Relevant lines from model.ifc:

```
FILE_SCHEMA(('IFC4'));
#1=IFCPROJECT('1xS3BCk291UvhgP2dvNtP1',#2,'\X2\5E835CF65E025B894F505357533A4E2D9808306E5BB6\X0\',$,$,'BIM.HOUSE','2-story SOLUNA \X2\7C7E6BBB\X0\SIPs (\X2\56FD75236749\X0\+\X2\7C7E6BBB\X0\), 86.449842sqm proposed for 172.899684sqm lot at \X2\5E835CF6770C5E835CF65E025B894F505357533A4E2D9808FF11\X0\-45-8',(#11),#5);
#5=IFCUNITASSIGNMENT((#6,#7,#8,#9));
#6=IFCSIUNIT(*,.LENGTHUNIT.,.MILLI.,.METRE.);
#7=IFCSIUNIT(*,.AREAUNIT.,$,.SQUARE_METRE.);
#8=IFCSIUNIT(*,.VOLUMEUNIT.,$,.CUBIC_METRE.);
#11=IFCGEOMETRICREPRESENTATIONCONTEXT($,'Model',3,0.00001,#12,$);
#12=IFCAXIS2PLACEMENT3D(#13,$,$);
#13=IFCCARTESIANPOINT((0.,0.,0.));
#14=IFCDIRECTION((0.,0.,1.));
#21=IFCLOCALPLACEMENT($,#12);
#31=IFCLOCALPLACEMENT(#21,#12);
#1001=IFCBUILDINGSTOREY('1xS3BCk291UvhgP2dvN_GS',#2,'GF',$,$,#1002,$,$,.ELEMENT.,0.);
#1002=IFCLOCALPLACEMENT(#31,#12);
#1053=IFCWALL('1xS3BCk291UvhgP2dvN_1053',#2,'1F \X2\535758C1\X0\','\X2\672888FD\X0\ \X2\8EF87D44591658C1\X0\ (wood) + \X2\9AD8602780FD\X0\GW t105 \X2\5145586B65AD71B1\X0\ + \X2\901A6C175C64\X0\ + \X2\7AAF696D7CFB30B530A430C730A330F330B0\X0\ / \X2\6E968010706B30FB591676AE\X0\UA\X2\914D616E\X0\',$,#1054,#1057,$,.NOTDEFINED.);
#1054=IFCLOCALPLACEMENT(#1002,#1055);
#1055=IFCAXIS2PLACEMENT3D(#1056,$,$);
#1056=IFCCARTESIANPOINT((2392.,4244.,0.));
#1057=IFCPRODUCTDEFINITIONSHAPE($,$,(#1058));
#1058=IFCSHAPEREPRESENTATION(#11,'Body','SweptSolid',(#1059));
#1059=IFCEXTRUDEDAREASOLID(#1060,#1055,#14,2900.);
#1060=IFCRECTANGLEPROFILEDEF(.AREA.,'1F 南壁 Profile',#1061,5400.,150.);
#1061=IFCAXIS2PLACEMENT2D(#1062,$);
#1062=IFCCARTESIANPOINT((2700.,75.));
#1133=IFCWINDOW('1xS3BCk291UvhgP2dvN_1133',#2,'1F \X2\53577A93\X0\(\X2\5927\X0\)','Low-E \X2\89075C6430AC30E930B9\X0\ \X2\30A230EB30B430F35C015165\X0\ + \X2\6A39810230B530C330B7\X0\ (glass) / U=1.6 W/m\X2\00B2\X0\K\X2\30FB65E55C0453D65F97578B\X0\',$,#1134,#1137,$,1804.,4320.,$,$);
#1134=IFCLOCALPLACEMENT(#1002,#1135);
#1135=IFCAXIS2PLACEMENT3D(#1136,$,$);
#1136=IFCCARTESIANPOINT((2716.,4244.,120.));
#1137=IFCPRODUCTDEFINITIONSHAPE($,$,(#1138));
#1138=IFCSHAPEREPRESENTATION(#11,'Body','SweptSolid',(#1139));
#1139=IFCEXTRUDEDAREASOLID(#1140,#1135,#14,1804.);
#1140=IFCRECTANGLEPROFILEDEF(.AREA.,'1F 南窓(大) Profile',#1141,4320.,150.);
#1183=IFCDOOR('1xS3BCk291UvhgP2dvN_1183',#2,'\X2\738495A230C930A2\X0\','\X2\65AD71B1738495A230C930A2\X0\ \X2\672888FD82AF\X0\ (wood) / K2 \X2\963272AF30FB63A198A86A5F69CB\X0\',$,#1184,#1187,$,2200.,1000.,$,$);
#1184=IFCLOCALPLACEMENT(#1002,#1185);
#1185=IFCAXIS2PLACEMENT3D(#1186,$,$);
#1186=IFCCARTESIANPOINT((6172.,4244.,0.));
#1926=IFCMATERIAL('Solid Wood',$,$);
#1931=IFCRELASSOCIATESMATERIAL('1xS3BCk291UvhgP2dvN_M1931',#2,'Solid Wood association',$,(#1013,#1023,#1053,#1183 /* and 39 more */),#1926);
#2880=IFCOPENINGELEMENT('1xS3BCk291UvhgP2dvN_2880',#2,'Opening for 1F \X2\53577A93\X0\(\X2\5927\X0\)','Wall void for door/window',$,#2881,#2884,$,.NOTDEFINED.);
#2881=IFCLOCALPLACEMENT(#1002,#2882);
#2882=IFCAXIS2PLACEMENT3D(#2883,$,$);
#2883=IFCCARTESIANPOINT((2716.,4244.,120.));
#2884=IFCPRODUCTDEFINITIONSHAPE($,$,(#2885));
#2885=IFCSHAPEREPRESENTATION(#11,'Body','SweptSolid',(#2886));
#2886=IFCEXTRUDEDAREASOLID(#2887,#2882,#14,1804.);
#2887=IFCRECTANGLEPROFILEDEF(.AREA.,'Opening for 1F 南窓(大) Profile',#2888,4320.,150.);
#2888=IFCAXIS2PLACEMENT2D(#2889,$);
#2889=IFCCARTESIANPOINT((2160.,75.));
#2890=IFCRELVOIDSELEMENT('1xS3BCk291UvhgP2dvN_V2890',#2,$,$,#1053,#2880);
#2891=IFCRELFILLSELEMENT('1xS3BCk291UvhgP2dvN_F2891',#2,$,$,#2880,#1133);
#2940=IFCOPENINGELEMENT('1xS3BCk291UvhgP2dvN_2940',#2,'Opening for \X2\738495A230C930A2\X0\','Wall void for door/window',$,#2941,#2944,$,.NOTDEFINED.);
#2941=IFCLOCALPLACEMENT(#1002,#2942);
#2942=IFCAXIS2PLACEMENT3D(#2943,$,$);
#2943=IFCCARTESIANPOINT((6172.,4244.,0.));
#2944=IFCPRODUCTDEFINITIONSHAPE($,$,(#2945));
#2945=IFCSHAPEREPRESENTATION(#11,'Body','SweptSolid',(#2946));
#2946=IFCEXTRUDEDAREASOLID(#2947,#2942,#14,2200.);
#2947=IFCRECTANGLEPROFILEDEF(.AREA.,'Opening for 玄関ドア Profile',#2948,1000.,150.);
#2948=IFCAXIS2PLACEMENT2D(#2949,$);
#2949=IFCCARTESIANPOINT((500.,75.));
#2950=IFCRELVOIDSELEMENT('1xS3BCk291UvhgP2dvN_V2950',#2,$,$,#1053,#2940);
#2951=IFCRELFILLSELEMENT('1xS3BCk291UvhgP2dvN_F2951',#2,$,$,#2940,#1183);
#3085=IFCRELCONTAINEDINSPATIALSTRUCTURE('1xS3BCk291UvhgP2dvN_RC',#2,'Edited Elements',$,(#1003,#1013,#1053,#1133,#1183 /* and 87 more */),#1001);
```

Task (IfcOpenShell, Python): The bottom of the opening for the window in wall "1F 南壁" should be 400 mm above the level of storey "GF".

```python
import numpy as np
import ifcopenshell
import ifcopenshell.api.geometry
import ifcopenshell.geom
import ifcopenshell.util.element
import ifcopenshell.util.placement
import ifcopenshell.util.shape
import ifcopenshell.util.unit

model = ifcopenshell.open("model.ifc")
unit_scale = ifcopenshell.util.unit.calculate_unit_scale(model)

window = model.by_guid("1xS3BCk291UvhgP2dvN_1133")
opening = window.FillsVoids[0].RelatingOpeningElement
storey = ifcopenshell.util.element.get_container(window, ifc_class="IfcBuildingStorey")
level = ifcopenshell.util.placement.get_local_placement(storey.ObjectPlacement)[2, 3]

# The opening's origin need not be at the sill, so measure its lowest point.
shape = ifcopenshell.geom.create_shape(ifcopenshell.geom.settings(), opening)
bottom = ifcopenshell.util.shape.get_shape_bottom_elevation(shape, shape.geometry) / unit_scale
dz = level + 400.0 - bottom

shift = np.array([0.0, 0.0, dz])
# The window is not placed relative to its opening, so move both.
for product in (opening, window):
    matrix = ifcopenshell.util.placement.get_local_placement(product.ObjectPlacement)
    matrix[:3, 3] += shift
    ifcopenshell.api.geometry.edit_object_placement(model, product=product, matrix=matrix, is_si=False)

print(f"moved by {dz * unit_scale:+.3f} m")

model.write("model_edited.ifc")
```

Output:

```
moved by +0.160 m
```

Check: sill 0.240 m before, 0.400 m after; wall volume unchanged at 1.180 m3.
